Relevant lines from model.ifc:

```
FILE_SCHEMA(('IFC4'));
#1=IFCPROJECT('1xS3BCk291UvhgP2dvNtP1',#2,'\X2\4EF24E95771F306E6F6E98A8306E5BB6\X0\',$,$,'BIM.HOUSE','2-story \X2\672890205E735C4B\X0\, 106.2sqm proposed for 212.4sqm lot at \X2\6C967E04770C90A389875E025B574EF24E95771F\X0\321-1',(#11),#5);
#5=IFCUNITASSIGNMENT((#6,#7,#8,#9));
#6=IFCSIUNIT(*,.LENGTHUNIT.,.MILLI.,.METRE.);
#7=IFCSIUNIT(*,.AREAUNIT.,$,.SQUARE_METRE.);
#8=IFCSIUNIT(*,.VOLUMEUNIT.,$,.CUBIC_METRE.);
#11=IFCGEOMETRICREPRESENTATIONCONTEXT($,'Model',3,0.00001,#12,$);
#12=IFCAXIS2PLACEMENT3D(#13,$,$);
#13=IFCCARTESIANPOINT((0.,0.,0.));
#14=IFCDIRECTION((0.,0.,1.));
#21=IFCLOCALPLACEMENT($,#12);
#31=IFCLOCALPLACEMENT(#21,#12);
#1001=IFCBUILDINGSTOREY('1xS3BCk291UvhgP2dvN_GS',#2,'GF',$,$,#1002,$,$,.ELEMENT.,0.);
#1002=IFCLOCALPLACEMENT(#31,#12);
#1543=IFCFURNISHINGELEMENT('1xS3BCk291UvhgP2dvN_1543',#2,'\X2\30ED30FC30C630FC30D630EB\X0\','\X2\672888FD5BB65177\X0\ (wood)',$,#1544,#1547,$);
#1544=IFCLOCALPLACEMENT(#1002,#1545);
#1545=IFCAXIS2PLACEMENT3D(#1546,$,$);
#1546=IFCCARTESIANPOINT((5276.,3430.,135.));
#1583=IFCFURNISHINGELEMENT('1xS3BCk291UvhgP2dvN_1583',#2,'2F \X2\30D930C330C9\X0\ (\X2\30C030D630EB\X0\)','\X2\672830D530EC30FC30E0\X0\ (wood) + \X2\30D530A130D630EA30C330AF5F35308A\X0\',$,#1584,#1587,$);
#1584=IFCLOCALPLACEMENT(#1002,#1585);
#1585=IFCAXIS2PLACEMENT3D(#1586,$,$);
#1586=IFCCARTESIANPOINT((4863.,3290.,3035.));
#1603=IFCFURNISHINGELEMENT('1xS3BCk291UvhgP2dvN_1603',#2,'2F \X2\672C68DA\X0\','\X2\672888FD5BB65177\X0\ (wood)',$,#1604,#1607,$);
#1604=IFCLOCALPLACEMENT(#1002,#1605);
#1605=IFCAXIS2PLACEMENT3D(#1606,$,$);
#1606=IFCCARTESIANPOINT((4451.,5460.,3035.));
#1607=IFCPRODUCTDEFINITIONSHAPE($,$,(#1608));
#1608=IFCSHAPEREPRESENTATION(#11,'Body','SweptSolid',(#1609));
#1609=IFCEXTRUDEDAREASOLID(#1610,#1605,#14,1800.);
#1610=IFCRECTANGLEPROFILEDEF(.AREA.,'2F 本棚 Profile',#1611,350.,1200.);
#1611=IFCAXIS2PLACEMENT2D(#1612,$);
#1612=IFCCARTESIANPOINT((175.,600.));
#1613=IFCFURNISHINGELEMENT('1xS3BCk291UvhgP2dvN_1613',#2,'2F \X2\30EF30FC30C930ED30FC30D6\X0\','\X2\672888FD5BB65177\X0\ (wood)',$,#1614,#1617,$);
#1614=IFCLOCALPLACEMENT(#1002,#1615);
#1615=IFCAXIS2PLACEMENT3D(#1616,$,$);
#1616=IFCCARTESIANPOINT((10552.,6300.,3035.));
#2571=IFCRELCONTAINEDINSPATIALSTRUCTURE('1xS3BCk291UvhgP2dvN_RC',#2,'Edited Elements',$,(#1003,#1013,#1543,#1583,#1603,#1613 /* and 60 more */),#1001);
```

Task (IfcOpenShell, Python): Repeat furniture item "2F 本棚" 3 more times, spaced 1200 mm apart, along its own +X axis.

```python
import ifcopenshell
import ifcopenshell.api.geometry
import ifcopenshell.api.root
import ifcopenshell.util.element
import ifcopenshell.util.placement
import ifcopenshell.util.unit

model = ifcopenshell.open("model.ifc")
unit_scale = ifcopenshell.util.unit.calculate_unit_scale(model)


def reuse_history(source, copy):
    """copy_class also copies each property set's owner history, people and application; keep the originals."""
    for rel in copy.IsDefinedBy:
        if rel.is_a("IfcRelDefinesByProperties") and (history := rel.RelatingPropertyDefinition.OwnerHistory):
            rel.RelatingPropertyDefinition.OwnerHistory = source.OwnerHistory
            ifcopenshell.util.element.remove_deep2(model, history)


source = model.by_guid("1xS3BCk291UvhgP2dvN_1603")
base = ifcopenshell.util.placement.get_local_placement(source.ObjectPlacement)
step = base[:3, 0] * 1.2 / unit_scale

for i in range(1, 4):
    copy = ifcopenshell.api.root.copy_class(model, product=source)
    copy.Representation = ifcopenshell.util.element.copy_deep(
        model, source.Representation, exclude=["IfcGeometricRepresentationContext", "IfcRepresentationMap"]
    )
    reuse_history(source, copy)
    matrix = base.copy()
    matrix[:3, 3] += i * step
    print("added at", matrix[:3, 3].round(3) + 0.0)
    ifcopenshell.api.geometry.edit_object_placement(model, product=copy, matrix=matrix, is_si=False)

model.write("model-out.ifc")
```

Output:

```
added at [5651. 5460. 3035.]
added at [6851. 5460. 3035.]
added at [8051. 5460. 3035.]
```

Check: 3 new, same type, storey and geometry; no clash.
